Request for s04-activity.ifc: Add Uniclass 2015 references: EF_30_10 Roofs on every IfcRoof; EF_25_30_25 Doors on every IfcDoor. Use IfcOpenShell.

First a look at what the model holds.

```python
import ifcopenshell

model = ifcopenshell.open("s04-activity.ifc")
print(model.schema)
print("classifications:", [c.Name for c in model.by_type("IfcClassification")])
for ifc_class in ("IfcDoor", "IfcRoof", "IfcStair", "IfcWall", "IfcWindow"):
    print(ifc_class, len(model.by_type(ifc_class)))
```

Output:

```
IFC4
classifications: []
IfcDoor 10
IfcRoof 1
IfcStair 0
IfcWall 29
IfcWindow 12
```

```python
import ifcopenshell
import ifcopenshell.api.classification

model = ifcopenshell.open("s04-activity.ifc")

system = ifcopenshell.api.classification.add_classification(model, classification="Uniclass 2015")

codes = {
    "IfcRoof": ("EF_30_10", "Roofs"),
    "IfcDoor": ("EF_25_30_25", "Doors"),
}
for ifc_class, (code, name) in codes.items():
    products = model.by_type(ifc_class)
    ifcopenshell.api.classification.add_reference(
        model, products=products, classification=system, identification=code, name=name
    )
    print(code, len(products))

model.write("s04-activity-out.ifc")
```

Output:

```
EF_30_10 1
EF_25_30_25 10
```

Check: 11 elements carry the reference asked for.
